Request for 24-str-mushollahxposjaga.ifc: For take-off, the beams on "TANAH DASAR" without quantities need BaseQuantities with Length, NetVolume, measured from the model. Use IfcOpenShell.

First a look at what the model holds.

```python
import ifcopenshell
import ifcopenshell.util.element
import ifcopenshell.util.unit

model = ifcopenshell.open("24-str-mushollahxposjaga.ifc")
print(model.schema)
for unit_type in ("LENGTHUNIT", "AREAUNIT", "VOLUMEUNIT"):
    print(unit_type, ifcopenshell.util.unit.calculate_unit_scale(model, unit_type))
storey = next(s for s in model.by_type("IfcBuildingStorey") if s.Name == "TANAH DASAR")
beams = [e for e in ifcopenshell.util.element.get_decomposition(storey) if e.is_a("IfcBeam")]
for e in sorted(beams, key=lambda e: e.id()):
    print(e.id(), e.is_a(), e.Name, list(ifcopenshell.util.element.get_psets(e, qtos_only=True)), sep=" | ")
```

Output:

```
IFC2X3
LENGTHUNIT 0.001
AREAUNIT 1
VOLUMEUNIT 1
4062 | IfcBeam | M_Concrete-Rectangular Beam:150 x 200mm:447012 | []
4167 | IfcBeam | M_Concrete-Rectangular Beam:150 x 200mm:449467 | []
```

```python
import ifcopenshell
import ifcopenshell.api.pset
import ifcopenshell.geom
import ifcopenshell.util.element
import ifcopenshell.util.shape
import ifcopenshell.util.unit

model = ifcopenshell.open("24-str-mushollahxposjaga.ifc")
unit_scale = ifcopenshell.util.unit.calculate_unit_scale(model)
volume_scale = ifcopenshell.util.unit.calculate_unit_scale(model, "VOLUMEUNIT")
settings = ifcopenshell.geom.settings()

storey = next(s for s in model.by_type("IfcBuildingStorey") if s.Name == "TANAH DASAR")
beams = [e for e in ifcopenshell.util.element.get_decomposition(storey) if e.is_a("IfcBeam")]

for e in sorted(beams, key=lambda e: e.id()):
    if ifcopenshell.util.element.get_psets(e, qtos_only=True, should_inherit=False):
        continue
    # Geometry comes back in metres, in the element's own axes.
    shape = ifcopenshell.geom.create_shape(settings, e)
    values = {
        "Length": ifcopenshell.util.shape.get_max_xyz(shape.geometry) / unit_scale,
        "NetVolume": ifcopenshell.util.shape.get_volume(shape.geometry) / volume_scale,
    }
    qto = ifcopenshell.api.pset.add_qto(model, product=e, name="BaseQuantities")
    ifcopenshell.api.pset.edit_qto(model, qto=qto, properties=values)
    print(e.id(), {k: round(v, 3) for k, v in values.items()})

model.write("24-str-mushollahxposjaga_v2.ifc")
```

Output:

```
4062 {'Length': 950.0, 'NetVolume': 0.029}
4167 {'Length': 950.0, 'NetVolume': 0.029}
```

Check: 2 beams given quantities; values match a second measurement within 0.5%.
